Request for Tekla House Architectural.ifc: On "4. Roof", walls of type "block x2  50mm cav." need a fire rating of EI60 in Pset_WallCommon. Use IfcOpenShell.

First a look at what the model holds.

```python
import ifcopenshell
import ifcopenshell.util.element

model = ifcopenshell.open("Tekla House Architectural.ifc")
print(model.schema)
storey = next(s for s in model.by_type("IfcBuildingStorey") if s.Name == "4. Roof")
walls = [e for e in ifcopenshell.util.element.get_decomposition(storey) if e.is_a("IfcWall")]
seen = {}
for e in walls:
    element_type = ifcopenshell.util.element.get_type(e)
    key = (element_type.Name if element_type != e and element_type else None, ifcopenshell.util.element.get_pset(e, "Pset_WallCommon", "FireRating"))
    seen[key] = seen.get(key, 0) + 1
for (name, value), count in sorted(seen.items(), key=str):
    print(count, "x", name, "|", value)
```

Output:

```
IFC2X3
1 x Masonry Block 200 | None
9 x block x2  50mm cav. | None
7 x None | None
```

```python
import ifcopenshell
import ifcopenshell.api.pset
import ifcopenshell.util.element

model = ifcopenshell.open("Tekla House Architectural.ifc")

storey = next(s for s in model.by_type("IfcBuildingStorey") if s.Name == "4. Roof")
walls = [e for e in ifcopenshell.util.element.get_decomposition(storey) if e.is_a("IfcWall")]

count = 0
for e in walls:
    element_type = ifcopenshell.util.element.get_type(e)
    if element_type in (None, e) or element_type.Name != "block x2  50mm cav.":
        continue
    # add_pset returns the element's existing set when there is one.
    pset = ifcopenshell.api.pset.add_pset(model, product=e, name="Pset_WallCommon")
    ifcopenshell.api.pset.edit_pset(model, pset=pset, properties={"FireRating": "EI60"})
    count += 1

print(count, "walls updated")

model.write("Tekla House Architectural-out.ifc")
```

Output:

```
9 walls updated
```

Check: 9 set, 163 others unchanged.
